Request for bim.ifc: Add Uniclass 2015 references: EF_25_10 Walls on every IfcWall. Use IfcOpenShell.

First a look at what the model holds.

```python
import ifcopenshell

model = ifcopenshell.open("bim.ifc")
print(model.schema)
print("classifications:", [c.Name for c in model.by_type("IfcClassification")])
for ifc_class in ("IfcDoor", "IfcRoof", "IfcStair", "IfcWall", "IfcWindow"):
    print(ifc_class, len(model.by_type(ifc_class)))
```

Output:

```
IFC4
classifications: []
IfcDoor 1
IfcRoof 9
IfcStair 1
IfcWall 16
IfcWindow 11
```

```python
import ifcopenshell
import ifcopenshell.api.classification

model = ifcopenshell.open("bim.ifc")

system = ifcopenshell.api.classification.add_classification(model, classification="Uniclass 2015")

codes = {
    "IfcWall": ("EF_25_10", "Walls"),
}
for ifc_class, (code, name) in codes.items():
    products = model.by_type(ifc_class)
    ifcopenshell.api.classification.add_reference(
        model, products=products, classification=system, identification=code, name=name
    )
    print(code, len(products))

model.write("bim_edited.ifc")
```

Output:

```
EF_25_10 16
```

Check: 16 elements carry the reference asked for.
